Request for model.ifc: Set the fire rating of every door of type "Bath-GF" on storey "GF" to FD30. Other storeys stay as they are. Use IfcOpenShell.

First a look at what the model holds.

```python
import ifcopenshell
import ifcopenshell.util.element

model = ifcopenshell.open("model.ifc")
print(model.schema)
storey = next(s for s in model.by_type("IfcBuildingStorey") if s.Name == "GF")
doors = [e for e in ifcopenshell.util.element.get_decomposition(storey) if e.is_a("IfcDoor")]
seen = {}
for e in doors:
    element_type = ifcopenshell.util.element.get_type(e)
    key = (element_type.Name if element_type != e and element_type else None, ifcopenshell.util.element.get_pset(e, "Pset_DoorCommon", "FireRating"))
    seen[key] = seen.get(key, 0) + 1
for (name, value), count in sorted(seen.items(), key=str):
    print(count, "x", name, "|", value)
```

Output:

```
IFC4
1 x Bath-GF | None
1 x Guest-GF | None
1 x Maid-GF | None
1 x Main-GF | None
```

```python
import ifcopenshell
import ifcopenshell.api.pset
import ifcopenshell.util.element

model = ifcopenshell.open("model.ifc")

storey = next(s for s in model.by_type("IfcBuildingStorey") if s.Name == "GF")
doors = [e for e in ifcopenshell.util.element.get_decomposition(storey) if e.is_a("IfcDoor")]

count = 0
for e in doors:
    element_type = ifcopenshell.util.element.get_type(e)
    if element_type in (None, e) or element_type.Name != "Bath-GF":
        continue
    # add_pset returns the element's existing set when there is one.
    pset = ifcopenshell.api.pset.add_pset(model, product=e, name="Pset_DoorCommon")
    ifcopenshell.api.pset.edit_pset(model, pset=pset, properties={"FireRating": "FD30"})
    count += 1

print(count, "doors updated")

model.write("model-out.ifc")
```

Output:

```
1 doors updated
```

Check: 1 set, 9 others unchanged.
